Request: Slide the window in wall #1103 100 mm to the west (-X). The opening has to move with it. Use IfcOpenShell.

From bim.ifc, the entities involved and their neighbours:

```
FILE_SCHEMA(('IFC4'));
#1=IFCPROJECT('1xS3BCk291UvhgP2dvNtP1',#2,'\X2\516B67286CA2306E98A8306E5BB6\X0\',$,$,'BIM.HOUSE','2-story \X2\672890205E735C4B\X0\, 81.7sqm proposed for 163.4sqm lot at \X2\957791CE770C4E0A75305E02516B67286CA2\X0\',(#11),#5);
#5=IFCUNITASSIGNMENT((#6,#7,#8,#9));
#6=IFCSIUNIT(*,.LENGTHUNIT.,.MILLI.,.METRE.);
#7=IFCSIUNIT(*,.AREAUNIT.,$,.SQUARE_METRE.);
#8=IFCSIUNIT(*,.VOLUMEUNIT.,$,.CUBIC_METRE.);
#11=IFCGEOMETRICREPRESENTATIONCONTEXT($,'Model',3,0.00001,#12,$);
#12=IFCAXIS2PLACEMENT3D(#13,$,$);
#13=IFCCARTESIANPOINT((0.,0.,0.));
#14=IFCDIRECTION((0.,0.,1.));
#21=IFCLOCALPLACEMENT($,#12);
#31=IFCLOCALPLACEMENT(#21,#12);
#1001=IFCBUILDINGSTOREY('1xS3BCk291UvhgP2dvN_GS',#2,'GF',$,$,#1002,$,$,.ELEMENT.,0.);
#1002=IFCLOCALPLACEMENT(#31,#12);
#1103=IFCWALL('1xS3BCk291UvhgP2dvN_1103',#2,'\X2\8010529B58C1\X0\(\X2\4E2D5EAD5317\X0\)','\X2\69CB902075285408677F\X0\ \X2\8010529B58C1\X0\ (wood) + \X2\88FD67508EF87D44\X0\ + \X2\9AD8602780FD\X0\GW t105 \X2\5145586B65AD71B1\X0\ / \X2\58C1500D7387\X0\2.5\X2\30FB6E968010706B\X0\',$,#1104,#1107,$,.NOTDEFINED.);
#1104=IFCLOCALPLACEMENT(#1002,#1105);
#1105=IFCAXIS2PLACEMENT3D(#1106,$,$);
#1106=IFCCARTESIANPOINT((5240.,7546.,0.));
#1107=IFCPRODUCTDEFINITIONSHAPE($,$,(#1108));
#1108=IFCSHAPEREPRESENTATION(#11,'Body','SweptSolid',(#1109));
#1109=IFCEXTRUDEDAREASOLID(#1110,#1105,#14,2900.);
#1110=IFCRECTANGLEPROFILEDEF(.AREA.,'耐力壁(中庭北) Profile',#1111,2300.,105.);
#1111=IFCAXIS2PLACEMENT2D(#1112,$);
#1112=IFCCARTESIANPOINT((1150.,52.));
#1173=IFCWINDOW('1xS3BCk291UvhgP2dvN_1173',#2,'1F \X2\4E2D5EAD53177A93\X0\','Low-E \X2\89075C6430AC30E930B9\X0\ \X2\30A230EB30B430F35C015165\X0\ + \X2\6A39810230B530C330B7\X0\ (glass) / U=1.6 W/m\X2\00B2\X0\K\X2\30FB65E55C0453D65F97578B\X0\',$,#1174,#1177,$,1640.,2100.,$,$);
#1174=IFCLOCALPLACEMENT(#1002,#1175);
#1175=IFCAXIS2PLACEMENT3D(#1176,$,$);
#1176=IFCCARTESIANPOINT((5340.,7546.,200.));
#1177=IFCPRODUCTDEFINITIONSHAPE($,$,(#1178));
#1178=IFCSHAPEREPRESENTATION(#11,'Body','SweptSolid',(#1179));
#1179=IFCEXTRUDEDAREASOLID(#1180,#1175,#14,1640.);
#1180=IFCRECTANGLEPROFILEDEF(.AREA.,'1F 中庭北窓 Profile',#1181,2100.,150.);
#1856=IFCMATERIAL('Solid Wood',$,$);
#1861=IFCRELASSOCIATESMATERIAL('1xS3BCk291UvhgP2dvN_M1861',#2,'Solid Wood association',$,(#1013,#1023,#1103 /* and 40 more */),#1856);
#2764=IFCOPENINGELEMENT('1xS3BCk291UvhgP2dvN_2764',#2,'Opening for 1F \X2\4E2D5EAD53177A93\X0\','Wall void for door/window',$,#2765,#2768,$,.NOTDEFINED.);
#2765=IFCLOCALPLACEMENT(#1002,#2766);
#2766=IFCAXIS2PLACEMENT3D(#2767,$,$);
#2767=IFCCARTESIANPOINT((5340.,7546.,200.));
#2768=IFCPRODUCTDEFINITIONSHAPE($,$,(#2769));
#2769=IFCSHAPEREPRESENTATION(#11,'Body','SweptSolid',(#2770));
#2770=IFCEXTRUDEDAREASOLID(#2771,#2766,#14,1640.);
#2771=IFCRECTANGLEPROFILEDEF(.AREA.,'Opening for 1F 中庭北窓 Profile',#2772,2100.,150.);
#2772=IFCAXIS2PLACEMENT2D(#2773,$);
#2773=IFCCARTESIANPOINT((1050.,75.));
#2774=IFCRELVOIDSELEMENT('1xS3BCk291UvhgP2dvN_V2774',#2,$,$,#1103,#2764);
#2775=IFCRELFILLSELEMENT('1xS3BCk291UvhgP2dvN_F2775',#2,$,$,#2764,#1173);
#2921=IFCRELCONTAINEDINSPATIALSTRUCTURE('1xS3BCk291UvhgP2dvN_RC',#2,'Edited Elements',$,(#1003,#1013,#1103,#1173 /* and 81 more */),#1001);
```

```python
import ifcopenshell
import ifcopenshell.api.geometry
import ifcopenshell.util.placement

model = ifcopenshell.open("bim.ifc")

window = model.by_id(1173)
opening = window.FillsVoids[0].RelatingOpeningElement
wall = opening.VoidsElements[0].RelatingBuildingElement

wall_matrix = ifcopenshell.util.placement.get_local_placement(wall.ObjectPlacement)
shift = wall_matrix[:3, 0] * -100.0
before = ifcopenshell.util.placement.get_local_placement(window.ObjectPlacement)[:3, 3].copy()

# The window is not placed relative to its opening, so move both.
for product in (opening, window):
    matrix = ifcopenshell.util.placement.get_local_placement(product.ObjectPlacement)
    matrix[:3, 3] += shift
    ifcopenshell.api.geometry.edit_object_placement(model, product=product, matrix=matrix, is_si=False)

after = ifcopenshell.util.placement.get_local_placement(window.ObjectPlacement)[:3, 3]
print("window moved by", (after - before).round(3) + 0.0)

model.write("bim_rev.ifc")
```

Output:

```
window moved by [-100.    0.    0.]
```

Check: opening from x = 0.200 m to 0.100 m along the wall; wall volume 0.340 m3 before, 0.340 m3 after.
